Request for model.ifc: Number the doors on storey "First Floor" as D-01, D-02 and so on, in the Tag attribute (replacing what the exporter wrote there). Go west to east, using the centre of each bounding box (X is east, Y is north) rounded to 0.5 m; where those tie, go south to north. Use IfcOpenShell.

First a look at what the model holds.

```python
import ifcopenshell
import ifcopenshell.util.element
import ifcopenshell.util.placement

model = ifcopenshell.open("model.ifc")
print(model.schema)
storey = next(s for s in model.by_type("IfcBuildingStorey") if s.Name == "First Floor")
doors = [e for e in ifcopenshell.util.element.get_decomposition(storey) if e.is_a("IfcDoor")]
for e in sorted(doors, key=lambda e: e.id()):
    origin = ifcopenshell.util.placement.get_local_placement(e.ObjectPlacement)[:3, 3]
    print(e.id(), e.Tag, e.Name, origin.round(2) + 0.0, sep=" | ")
```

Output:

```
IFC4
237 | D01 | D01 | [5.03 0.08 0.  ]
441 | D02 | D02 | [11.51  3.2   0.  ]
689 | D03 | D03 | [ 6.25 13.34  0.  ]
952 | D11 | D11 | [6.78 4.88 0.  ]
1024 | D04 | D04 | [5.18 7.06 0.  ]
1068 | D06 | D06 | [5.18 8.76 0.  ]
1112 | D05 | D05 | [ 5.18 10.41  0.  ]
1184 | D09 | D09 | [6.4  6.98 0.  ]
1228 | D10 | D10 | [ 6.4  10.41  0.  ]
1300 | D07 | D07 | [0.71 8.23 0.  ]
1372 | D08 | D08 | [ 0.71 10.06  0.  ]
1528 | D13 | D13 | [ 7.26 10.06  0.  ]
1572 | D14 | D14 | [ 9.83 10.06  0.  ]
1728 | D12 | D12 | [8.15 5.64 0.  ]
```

```python
import ifcopenshell
import ifcopenshell.geom
import ifcopenshell.util.element
import ifcopenshell.util.shape

model = ifcopenshell.open("model.ifc")
settings = ifcopenshell.geom.settings()
settings.set("use-world-coords", True)


def centre(element):
    shape = ifcopenshell.geom.create_shape(settings, element)
    return ifcopenshell.util.shape.get_bbox_centroid(shape.geometry)


storey = next(s for s in model.by_type("IfcBuildingStorey") if s.Name == "First Floor")
doors = [e for e in ifcopenshell.util.element.get_decomposition(storey) if e.is_a("IfcDoor")]

# Insertion points can sit at a corner or the storey origin, so sort by the geometry (in metres).
centres = {e: centre(e) for e in doors}
doors.sort(key=lambda e: (round(centres[e][0] / 0.5), centres[e][1]))

for i, e in enumerate(doors, start=1):
    number = f"D-{i:02d}"
    e.Tag = number
    print(e.id(), number)

model.write("model_v2.ifc")
```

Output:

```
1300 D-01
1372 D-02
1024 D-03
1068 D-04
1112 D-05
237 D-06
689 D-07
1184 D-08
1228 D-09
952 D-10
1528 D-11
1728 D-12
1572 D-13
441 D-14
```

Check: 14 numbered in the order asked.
